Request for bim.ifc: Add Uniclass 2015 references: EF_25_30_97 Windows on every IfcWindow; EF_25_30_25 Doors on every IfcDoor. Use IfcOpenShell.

First a look at what the model holds.

```python
import ifcopenshell

model = ifcopenshell.open("bim.ifc")
print(model.schema)
print("classifications:", [c.Name for c in model.by_type("IfcClassification")])
for ifc_class in ("IfcDoor", "IfcRoof", "IfcStair", "IfcWall", "IfcWindow"):
    print(ifc_class, len(model.by_type(ifc_class)))
```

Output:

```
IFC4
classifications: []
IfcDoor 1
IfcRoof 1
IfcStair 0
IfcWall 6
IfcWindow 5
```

```python
import ifcopenshell
import ifcopenshell.api.classification

model = ifcopenshell.open("bim.ifc")

system = ifcopenshell.api.classification.add_classification(model, classification="Uniclass 2015")

codes = {
    "IfcWindow": ("EF_25_30_97", "Windows"),
    "IfcDoor": ("EF_25_30_25", "Doors"),
}
for ifc_class, (code, name) in codes.items():
    products = model.by_type(ifc_class)
    ifcopenshell.api.classification.add_reference(
        model, products=products, classification=system, identification=code, name=name
    )
    print(code, len(products))

model.write("bim_rev.ifc")
```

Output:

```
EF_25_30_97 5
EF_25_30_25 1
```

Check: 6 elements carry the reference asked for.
